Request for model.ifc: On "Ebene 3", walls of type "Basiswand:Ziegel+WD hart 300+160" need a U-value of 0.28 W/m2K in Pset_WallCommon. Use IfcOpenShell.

First a look at what the model holds.

```python
import ifcopenshell
import ifcopenshell.util.element

model = ifcopenshell.open("model.ifc")
print(model.schema)
storey = next(s for s in model.by_type("IfcBuildingStorey") if s.Name == "Ebene 3")
walls = [e for e in ifcopenshell.util.element.get_decomposition(storey) if e.is_a("IfcWall")]
seen = {}
for e in walls:
    element_type = ifcopenshell.util.element.get_type(e)
    key = (element_type.Name if element_type != e and element_type else None, ifcopenshell.util.element.get_pset(e, "Pset_WallCommon", "ThermalTransmittance"))
    seen[key] = seen.get(key, 0) + 1
for (name, value), count in sorted(seen.items(), key=str):
    print(count, "x", name, "|", value)
```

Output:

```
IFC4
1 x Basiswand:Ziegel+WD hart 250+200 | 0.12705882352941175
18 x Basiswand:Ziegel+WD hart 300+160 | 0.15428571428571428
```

```python
import ifcopenshell
import ifcopenshell.api.pset
import ifcopenshell.util.element

model = ifcopenshell.open("model.ifc")

storey = next(s for s in model.by_type("IfcBuildingStorey") if s.Name == "Ebene 3")
walls = [e for e in ifcopenshell.util.element.get_decomposition(storey) if e.is_a("IfcWall")]

count = 0
for e in walls:
    element_type = ifcopenshell.util.element.get_type(e)
    if element_type in (None, e) or element_type.Name != "Basiswand:Ziegel+WD hart 300+160":
        continue
    # add_pset returns the element's existing set when there is one.
    pset = ifcopenshell.api.pset.add_pset(model, product=e, name="Pset_WallCommon")
    ifcopenshell.api.pset.edit_pset(model, pset=pset, properties={"ThermalTransmittance": 0.28})
    count += 1

print(count, "walls updated")

model.write("model_updated.ifc")
```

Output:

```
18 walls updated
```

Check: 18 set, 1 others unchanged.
